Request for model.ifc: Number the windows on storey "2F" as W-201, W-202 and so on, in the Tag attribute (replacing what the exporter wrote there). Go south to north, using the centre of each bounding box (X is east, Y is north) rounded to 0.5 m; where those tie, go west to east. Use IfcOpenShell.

First a look at what the model holds.

```python
import ifcopenshell
import ifcopenshell.util.element
import ifcopenshell.util.placement

model = ifcopenshell.open("model.ifc")
print(model.schema)
storey = next(s for s in model.by_type("IfcBuildingStorey") if s.Name == "2F")
windows = [e for e in ifcopenshell.util.element.get_decomposition(storey) if e.is_a("IfcWindow")]
for e in sorted(windows, key=lambda e: e.id()):
    origin = ifcopenshell.util.placement.get_local_placement(e.ObjectPlacement)[:3, 3]
    print(e.id(), e.Tag, e.Name, origin.round(2) + 0.0, sep=" | ")
```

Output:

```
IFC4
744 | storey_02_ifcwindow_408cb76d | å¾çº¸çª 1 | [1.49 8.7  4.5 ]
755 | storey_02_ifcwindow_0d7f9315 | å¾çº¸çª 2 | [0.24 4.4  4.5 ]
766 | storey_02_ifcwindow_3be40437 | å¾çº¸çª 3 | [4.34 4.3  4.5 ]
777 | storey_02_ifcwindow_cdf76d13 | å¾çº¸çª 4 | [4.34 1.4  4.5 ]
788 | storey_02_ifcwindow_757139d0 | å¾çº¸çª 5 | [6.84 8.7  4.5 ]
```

```python
import ifcopenshell
import ifcopenshell.geom
import ifcopenshell.util.element
import ifcopenshell.util.shape

model = ifcopenshell.open("model.ifc")
settings = ifcopenshell.geom.settings()
settings.set("use-world-coords", True)


def centre(element):
    shape = ifcopenshell.geom.create_shape(settings, element)
    return ifcopenshell.util.shape.get_bbox_centroid(shape.geometry)


storey = next(s for s in model.by_type("IfcBuildingStorey") if s.Name == "2F")
windows = [e for e in ifcopenshell.util.element.get_decomposition(storey) if e.is_a("IfcWindow")]

# Insertion points can sit at a corner or the storey origin, so sort by the geometry (in metres).
centres = {e: centre(e) for e in windows}
windows.sort(key=lambda e: (round(centres[e][1] / 0.5), centres[e][0]))

for i, e in enumerate(windows, start=1):
    number = f"W-2{i:02d}"
    e.Tag = number
    print(e.id(), number)

model.write("model_updated.ifc")
```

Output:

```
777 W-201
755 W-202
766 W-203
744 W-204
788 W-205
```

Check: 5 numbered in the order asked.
